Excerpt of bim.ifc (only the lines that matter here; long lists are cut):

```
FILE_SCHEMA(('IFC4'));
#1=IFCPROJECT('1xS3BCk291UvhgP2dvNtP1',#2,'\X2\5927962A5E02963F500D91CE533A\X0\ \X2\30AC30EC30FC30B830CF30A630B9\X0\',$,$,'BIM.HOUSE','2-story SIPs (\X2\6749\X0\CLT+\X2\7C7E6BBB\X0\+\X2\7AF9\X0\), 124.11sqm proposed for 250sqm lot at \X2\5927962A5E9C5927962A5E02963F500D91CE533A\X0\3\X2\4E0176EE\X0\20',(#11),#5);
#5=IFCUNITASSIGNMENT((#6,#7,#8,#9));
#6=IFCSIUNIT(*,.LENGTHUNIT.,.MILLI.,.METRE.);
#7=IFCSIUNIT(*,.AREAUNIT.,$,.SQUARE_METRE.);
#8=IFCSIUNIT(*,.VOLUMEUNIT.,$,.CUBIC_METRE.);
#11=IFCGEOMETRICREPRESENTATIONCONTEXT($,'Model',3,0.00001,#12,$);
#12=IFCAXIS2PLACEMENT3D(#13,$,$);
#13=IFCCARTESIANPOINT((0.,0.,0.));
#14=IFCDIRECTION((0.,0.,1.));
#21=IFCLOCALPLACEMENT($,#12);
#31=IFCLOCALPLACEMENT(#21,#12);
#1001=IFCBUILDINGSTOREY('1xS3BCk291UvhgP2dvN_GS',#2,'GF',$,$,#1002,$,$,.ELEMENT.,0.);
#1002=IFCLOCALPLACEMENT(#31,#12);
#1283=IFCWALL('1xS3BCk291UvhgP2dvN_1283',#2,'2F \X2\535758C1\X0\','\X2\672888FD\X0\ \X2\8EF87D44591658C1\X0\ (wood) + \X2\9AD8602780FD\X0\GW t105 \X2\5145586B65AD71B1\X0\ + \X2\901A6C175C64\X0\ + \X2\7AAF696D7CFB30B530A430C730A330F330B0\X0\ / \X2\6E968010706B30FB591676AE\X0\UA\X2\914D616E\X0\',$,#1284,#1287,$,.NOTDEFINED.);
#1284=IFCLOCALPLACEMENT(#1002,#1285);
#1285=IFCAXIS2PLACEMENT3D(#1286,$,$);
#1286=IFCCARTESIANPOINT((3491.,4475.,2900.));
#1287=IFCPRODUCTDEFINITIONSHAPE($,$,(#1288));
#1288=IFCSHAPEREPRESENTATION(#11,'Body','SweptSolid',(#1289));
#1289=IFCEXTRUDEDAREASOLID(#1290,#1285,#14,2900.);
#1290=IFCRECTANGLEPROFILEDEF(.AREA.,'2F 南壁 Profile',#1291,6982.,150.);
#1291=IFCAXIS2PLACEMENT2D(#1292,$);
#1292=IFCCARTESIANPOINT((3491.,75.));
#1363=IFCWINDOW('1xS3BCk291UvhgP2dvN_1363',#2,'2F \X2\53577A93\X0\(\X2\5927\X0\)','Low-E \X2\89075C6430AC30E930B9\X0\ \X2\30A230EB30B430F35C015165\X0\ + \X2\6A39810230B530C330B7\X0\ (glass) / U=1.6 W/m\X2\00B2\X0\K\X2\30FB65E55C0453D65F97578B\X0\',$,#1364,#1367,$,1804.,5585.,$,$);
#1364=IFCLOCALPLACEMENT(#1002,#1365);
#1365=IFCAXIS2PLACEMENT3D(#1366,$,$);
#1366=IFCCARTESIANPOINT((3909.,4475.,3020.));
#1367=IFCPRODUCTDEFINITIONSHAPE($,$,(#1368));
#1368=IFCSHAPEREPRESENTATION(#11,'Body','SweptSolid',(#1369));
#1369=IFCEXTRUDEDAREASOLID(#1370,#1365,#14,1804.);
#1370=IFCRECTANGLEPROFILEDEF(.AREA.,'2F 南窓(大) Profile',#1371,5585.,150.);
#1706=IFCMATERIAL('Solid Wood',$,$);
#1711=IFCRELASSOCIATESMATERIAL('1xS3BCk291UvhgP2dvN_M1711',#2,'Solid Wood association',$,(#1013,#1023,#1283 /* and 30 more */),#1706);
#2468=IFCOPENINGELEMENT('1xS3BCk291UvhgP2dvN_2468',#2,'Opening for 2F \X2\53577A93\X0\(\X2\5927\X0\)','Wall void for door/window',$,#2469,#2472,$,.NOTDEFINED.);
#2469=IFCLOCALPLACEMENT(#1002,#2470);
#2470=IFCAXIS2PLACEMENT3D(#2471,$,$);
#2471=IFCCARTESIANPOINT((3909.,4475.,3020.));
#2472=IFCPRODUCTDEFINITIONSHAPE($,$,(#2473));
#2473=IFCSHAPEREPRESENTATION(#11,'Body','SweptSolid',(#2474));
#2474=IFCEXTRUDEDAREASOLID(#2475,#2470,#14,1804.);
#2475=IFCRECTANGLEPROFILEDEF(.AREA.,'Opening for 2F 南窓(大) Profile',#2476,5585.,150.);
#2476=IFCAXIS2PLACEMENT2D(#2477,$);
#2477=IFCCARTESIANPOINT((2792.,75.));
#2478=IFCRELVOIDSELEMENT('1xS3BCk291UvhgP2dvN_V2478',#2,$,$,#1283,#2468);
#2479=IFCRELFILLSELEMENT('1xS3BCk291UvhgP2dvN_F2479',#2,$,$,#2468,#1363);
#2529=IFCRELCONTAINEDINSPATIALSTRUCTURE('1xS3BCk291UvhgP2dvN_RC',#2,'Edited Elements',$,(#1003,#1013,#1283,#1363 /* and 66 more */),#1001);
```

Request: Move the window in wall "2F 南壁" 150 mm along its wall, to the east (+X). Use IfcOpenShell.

```python
import ifcopenshell
import ifcopenshell.api.geometry
import ifcopenshell.util.placement
import ifcopenshell.util.unit

model = ifcopenshell.open("bim.ifc")
unit_scale = ifcopenshell.util.unit.calculate_unit_scale(model)

window = model.by_id(1363)
opening = window.FillsVoids[0].RelatingOpeningElement
wall = opening.VoidsElements[0].RelatingBuildingElement

wall_matrix = ifcopenshell.util.placement.get_local_placement(wall.ObjectPlacement)
shift = wall_matrix[:3, 0] * 0.15 / unit_scale
before = ifcopenshell.util.placement.get_local_placement(window.ObjectPlacement)[:3, 3].copy()

# The window is not placed relative to its opening, so move both.
for product in (opening, window):
    matrix = ifcopenshell.util.placement.get_local_placement(product.ObjectPlacement)
    matrix[:3, 3] += shift
    ifcopenshell.api.geometry.edit_object_placement(model, product=product, matrix=matrix, is_si=False)

after = ifcopenshell.util.placement.get_local_placement(window.ObjectPlacement)[:3, 3]
print("window moved by", (after - before).round(3) + 0.0)

model.write("bim-out.ifc")
```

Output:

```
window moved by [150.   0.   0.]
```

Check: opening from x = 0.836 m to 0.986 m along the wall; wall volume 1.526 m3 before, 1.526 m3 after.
